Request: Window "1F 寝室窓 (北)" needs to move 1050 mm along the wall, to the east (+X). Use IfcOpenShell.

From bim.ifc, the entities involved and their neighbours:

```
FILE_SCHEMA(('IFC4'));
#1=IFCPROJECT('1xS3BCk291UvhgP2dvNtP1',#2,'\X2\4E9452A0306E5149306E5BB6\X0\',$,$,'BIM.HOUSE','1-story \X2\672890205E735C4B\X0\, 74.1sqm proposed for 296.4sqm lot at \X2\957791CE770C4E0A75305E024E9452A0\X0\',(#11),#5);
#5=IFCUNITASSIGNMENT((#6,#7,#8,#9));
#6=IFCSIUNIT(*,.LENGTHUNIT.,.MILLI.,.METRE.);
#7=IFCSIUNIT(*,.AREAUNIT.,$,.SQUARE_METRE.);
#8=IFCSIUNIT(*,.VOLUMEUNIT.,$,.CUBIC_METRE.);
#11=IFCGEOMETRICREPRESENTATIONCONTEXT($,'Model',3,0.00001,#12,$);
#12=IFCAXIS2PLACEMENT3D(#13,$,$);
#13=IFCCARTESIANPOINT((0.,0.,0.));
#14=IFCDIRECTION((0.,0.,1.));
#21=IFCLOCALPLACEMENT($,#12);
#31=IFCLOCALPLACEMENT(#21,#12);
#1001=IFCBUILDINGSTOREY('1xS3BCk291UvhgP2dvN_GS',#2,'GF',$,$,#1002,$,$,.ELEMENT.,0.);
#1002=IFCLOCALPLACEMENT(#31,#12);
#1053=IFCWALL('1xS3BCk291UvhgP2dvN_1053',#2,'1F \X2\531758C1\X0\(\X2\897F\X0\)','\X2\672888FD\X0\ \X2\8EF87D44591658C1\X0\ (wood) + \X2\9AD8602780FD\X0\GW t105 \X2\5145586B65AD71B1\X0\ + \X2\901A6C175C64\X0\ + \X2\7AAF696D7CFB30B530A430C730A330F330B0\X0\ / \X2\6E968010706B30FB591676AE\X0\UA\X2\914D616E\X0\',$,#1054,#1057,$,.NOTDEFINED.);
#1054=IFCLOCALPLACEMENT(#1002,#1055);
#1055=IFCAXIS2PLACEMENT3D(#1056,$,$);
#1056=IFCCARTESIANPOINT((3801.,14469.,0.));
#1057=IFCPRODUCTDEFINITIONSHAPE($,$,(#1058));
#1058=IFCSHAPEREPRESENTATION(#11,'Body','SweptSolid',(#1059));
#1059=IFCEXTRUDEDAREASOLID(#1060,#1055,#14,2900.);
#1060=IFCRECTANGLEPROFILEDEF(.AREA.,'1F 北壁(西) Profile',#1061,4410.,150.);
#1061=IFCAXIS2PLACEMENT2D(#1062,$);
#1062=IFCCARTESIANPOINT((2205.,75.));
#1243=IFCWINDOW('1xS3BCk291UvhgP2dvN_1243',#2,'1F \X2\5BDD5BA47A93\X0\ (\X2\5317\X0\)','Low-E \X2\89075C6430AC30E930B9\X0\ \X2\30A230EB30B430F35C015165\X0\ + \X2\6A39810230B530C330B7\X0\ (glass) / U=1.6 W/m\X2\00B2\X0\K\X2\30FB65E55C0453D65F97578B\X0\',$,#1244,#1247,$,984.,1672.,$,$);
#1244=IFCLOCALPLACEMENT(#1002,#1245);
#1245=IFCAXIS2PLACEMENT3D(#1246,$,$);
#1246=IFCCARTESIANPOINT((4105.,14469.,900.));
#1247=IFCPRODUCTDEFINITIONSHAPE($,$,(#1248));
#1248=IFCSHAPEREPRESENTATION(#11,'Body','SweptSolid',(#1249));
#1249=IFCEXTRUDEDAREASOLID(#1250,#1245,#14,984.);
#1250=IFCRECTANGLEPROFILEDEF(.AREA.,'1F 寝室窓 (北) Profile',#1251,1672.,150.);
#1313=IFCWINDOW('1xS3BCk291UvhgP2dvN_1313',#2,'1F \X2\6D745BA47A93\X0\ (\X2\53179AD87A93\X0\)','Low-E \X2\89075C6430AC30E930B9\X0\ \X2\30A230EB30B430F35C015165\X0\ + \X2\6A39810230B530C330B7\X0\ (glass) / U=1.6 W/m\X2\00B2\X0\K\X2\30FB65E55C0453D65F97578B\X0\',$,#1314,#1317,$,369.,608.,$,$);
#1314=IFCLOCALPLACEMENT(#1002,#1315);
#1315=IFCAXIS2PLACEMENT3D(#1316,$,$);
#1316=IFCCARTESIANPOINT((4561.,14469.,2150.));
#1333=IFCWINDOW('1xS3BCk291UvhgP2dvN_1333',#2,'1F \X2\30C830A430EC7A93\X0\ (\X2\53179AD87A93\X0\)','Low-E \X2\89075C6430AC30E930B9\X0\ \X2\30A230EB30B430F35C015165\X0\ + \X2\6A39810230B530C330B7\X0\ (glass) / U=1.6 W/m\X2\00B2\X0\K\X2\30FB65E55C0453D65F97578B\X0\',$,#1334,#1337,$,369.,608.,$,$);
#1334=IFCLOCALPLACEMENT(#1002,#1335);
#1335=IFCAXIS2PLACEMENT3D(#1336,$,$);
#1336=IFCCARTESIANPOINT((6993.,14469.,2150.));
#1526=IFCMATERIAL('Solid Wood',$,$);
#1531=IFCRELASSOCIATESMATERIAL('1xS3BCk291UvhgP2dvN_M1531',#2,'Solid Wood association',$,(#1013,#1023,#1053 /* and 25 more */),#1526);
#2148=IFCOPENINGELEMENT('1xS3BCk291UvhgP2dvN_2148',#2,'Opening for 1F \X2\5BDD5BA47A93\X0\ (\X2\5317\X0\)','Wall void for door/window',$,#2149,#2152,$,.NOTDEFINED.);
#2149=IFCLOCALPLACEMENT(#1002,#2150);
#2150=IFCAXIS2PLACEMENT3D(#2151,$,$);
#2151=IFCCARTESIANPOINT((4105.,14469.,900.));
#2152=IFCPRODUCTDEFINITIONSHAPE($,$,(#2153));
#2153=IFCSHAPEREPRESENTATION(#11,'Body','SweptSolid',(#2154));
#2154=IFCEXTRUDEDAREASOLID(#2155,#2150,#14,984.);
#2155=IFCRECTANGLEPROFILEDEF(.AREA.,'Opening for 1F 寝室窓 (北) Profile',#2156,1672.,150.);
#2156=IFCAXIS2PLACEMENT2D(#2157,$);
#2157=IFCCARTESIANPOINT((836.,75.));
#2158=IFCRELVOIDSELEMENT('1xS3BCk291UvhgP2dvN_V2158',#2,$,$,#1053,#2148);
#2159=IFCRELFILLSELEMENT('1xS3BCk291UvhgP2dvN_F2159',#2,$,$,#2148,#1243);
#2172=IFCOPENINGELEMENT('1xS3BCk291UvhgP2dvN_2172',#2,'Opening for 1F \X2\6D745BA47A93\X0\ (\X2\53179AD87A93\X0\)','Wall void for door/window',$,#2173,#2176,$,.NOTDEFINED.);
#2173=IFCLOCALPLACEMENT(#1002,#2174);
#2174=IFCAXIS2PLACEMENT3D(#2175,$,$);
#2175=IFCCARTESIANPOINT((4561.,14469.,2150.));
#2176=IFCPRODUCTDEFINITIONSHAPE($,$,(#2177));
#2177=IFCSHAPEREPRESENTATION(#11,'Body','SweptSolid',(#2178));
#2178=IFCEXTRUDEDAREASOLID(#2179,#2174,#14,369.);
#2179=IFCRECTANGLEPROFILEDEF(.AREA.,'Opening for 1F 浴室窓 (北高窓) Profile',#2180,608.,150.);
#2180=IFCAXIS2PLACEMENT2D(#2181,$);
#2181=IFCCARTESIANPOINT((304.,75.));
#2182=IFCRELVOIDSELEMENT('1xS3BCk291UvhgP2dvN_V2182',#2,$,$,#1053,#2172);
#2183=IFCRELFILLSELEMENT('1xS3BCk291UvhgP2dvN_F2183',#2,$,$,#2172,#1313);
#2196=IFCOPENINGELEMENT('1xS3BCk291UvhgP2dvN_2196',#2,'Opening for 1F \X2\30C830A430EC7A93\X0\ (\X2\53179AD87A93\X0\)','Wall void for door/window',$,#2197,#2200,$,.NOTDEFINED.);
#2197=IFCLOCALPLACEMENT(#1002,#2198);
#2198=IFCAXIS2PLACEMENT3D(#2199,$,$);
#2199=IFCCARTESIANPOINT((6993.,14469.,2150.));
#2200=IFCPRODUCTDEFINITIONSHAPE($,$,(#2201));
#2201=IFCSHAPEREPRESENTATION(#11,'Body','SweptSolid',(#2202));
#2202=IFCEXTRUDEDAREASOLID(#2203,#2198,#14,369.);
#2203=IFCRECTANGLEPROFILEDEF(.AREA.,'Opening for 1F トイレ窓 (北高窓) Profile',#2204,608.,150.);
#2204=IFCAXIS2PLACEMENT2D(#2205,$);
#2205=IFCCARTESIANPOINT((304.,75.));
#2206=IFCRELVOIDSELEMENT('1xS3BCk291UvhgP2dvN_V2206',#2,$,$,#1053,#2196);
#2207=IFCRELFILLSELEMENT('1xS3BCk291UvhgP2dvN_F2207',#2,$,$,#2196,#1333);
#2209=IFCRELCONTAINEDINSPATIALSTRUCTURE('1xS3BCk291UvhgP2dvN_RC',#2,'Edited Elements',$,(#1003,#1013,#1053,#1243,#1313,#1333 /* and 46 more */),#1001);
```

```python
import ifcopenshell
import ifcopenshell.api.geometry
import ifcopenshell.util.placement

model = ifcopenshell.open("bim.ifc")

window = model.by_guid("1xS3BCk291UvhgP2dvN_1243")
opening = window.FillsVoids[0].RelatingOpeningElement
wall = opening.VoidsElements[0].RelatingBuildingElement

wall_matrix = ifcopenshell.util.placement.get_local_placement(wall.ObjectPlacement)
shift = wall_matrix[:3, 0] * 1050.0
before = ifcopenshell.util.placement.get_local_placement(window.ObjectPlacement)[:3, 3].copy()

# The window is not placed relative to its opening, so move both.
for product in (opening, window):
    matrix = ifcopenshell.util.placement.get_local_placement(product.ObjectPlacement)
    matrix[:3, 3] += shift
    ifcopenshell.api.geometry.edit_object_placement(model, product=product, matrix=matrix, is_si=False)

after = ifcopenshell.util.placement.get_local_placement(window.ObjectPlacement)[:3, 3]
print("window moved by", (after - before).round(3) + 0.0)

model.write("bim-out.ifc")
```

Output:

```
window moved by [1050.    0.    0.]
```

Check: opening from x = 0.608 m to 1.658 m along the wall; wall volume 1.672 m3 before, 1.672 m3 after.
